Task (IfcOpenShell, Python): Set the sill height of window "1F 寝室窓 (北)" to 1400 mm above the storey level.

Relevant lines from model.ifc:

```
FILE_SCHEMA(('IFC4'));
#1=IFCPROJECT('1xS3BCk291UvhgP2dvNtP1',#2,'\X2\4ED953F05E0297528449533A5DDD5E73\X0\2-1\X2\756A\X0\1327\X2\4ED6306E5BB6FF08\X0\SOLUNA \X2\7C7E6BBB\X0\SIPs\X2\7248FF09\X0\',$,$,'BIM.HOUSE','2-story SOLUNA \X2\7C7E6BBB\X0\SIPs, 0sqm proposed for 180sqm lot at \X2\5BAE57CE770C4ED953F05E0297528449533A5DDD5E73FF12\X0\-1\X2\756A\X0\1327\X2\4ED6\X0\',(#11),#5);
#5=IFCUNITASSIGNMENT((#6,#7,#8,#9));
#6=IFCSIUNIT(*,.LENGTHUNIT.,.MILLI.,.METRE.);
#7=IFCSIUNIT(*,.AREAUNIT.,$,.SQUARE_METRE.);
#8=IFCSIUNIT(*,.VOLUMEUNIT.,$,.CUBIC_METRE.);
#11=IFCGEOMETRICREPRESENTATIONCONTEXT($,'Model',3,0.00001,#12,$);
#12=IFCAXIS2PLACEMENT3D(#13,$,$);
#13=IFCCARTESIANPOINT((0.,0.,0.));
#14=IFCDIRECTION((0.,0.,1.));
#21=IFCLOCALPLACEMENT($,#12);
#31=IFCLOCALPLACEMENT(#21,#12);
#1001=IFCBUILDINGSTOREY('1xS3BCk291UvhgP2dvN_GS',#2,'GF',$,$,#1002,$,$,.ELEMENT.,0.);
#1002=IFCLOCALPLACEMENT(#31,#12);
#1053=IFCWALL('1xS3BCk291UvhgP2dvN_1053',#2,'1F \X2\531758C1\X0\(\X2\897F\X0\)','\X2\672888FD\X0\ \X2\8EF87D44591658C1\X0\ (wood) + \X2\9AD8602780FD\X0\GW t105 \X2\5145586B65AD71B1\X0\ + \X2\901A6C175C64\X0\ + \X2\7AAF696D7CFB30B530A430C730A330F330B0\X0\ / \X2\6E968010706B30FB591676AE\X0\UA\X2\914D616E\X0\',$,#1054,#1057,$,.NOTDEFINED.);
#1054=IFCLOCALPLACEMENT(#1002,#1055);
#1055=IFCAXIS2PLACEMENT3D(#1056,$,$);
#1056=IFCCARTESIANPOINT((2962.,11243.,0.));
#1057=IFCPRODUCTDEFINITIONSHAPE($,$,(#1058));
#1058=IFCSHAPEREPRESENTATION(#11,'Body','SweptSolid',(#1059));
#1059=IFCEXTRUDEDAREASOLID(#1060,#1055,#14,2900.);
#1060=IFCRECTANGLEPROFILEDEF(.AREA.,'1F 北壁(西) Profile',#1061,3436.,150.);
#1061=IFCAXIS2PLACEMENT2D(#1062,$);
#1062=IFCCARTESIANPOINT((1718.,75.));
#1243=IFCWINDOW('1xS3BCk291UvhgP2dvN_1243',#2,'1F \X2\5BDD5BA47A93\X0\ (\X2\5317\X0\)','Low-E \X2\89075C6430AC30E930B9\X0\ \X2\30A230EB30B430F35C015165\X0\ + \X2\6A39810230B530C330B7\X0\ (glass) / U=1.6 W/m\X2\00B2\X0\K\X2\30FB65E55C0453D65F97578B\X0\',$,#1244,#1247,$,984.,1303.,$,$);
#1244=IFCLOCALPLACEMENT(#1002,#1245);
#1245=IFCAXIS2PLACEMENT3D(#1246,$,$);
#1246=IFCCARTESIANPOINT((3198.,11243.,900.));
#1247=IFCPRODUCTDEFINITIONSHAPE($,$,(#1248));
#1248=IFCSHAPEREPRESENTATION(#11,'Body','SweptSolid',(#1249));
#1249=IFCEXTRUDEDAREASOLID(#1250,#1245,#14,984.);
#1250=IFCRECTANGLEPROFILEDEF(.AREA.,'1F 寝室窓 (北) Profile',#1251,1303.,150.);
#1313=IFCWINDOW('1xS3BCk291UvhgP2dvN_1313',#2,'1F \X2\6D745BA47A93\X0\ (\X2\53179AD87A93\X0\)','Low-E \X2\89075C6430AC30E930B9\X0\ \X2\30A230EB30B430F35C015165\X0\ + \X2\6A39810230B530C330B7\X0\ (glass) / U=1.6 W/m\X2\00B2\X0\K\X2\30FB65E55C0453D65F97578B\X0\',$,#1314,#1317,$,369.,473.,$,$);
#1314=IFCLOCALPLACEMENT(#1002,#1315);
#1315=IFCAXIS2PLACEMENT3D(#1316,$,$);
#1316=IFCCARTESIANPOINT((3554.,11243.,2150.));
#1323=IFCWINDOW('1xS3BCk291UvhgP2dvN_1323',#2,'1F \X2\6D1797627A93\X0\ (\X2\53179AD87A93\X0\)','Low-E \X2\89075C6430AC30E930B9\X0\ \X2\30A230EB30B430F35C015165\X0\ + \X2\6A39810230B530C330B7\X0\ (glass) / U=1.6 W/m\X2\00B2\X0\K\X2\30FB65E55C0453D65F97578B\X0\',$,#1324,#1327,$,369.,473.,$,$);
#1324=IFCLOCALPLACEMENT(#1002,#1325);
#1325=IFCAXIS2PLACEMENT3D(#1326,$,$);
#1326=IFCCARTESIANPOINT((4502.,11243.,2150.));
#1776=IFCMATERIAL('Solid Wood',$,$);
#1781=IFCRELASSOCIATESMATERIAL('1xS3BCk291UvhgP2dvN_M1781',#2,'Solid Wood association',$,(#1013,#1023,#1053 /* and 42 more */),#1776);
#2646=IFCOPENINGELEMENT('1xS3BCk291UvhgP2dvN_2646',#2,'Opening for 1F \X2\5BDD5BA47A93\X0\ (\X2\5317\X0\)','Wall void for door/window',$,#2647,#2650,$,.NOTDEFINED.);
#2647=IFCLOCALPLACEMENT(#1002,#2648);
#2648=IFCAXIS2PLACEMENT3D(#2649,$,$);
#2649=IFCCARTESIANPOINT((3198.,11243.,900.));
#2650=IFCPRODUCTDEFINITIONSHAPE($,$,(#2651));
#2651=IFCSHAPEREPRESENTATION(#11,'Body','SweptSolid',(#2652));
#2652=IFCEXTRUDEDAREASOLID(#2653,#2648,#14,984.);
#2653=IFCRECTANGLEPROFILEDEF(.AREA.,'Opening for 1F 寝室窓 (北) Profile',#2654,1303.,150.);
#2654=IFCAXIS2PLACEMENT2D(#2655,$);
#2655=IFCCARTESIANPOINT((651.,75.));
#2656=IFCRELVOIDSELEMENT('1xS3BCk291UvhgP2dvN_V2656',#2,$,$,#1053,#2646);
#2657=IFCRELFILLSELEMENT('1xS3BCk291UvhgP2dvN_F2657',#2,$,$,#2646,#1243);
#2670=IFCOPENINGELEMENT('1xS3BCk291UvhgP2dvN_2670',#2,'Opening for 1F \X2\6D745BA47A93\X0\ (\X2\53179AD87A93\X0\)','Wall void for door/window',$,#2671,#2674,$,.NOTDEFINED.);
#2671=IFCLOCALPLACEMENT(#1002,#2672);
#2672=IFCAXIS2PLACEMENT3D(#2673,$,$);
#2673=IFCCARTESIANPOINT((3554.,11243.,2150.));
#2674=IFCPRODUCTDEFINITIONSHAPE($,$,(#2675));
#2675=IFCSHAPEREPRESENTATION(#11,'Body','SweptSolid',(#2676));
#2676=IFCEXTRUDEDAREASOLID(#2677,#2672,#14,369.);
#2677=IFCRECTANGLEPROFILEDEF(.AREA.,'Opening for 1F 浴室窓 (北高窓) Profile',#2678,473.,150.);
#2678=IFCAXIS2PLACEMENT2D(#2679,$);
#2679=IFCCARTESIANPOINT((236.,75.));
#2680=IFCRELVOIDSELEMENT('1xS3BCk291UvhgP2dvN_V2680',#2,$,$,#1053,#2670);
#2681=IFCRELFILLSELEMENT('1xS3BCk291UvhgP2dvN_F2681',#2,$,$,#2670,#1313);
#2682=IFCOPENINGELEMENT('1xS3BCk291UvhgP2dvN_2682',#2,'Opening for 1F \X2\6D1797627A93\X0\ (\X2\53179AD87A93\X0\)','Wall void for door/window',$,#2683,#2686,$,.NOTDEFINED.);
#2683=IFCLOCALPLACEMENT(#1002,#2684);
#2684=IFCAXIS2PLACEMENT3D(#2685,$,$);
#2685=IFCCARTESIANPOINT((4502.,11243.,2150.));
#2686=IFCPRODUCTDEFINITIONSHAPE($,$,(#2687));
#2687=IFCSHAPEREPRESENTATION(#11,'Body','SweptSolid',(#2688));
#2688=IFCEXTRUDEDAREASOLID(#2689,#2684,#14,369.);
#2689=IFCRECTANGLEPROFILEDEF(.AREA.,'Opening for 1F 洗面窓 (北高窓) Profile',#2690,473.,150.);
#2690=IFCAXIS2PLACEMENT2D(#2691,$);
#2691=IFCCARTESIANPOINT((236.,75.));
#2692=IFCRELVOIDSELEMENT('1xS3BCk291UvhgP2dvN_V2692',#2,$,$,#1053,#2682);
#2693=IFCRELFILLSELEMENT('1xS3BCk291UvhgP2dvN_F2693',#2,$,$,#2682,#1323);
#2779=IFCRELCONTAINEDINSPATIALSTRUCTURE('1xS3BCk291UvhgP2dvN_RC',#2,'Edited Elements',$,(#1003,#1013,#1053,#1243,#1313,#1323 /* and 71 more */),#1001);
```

```python
import numpy as np
import ifcopenshell
import ifcopenshell.api.geometry
import ifcopenshell.geom
import ifcopenshell.util.element
import ifcopenshell.util.placement
import ifcopenshell.util.shape
import ifcopenshell.util.unit

model = ifcopenshell.open("model.ifc")
unit_scale = ifcopenshell.util.unit.calculate_unit_scale(model)

window = model.by_guid("1xS3BCk291UvhgP2dvN_1243")
opening = window.FillsVoids[0].RelatingOpeningElement
storey = ifcopenshell.util.element.get_container(window, ifc_class="IfcBuildingStorey")
level = ifcopenshell.util.placement.get_local_placement(storey.ObjectPlacement)[2, 3]

# The opening's origin need not be at the sill, so measure its lowest point.
shape = ifcopenshell.geom.create_shape(ifcopenshell.geom.settings(), opening)
bottom = ifcopenshell.util.shape.get_shape_bottom_elevation(shape, shape.geometry) / unit_scale
dz = level + 1400.0 - bottom

shift = np.array([0.0, 0.0, dz])
# The window is not placed relative to its opening, so move both.
for product in (opening, window):
    matrix = ifcopenshell.util.placement.get_local_placement(product.ObjectPlacement)
    matrix[:3, 3] += shift
    ifcopenshell.api.geometry.edit_object_placement(model, product=product, matrix=matrix, is_si=False)

print(f"moved by {dz * unit_scale:+.3f} m")

model.write("model-out.ifc")
```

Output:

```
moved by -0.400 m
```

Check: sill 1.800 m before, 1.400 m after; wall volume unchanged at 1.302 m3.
